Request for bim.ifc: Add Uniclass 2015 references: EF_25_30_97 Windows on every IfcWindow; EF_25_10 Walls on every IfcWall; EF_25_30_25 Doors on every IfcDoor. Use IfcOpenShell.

First a look at what the model holds.

```python
import ifcopenshell

model = ifcopenshell.open("bim.ifc")
print(model.schema)
print("classifications:", [c.Name for c in model.by_type("IfcClassification")])
for ifc_class in ("IfcDoor", "IfcRoof", "IfcStair", "IfcWall", "IfcWindow"):
    print(ifc_class, len(model.by_type(ifc_class)))
```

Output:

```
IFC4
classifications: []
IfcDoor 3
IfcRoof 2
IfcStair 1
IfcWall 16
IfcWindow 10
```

```python
import ifcopenshell
import ifcopenshell.api.classification

model = ifcopenshell.open("bim.ifc")

system = ifcopenshell.api.classification.add_classification(model, classification="Uniclass 2015")

codes = {
    "IfcWindow": ("EF_25_30_97", "Windows"),
    "IfcWall": ("EF_25_10", "Walls"),
    "IfcDoor": ("EF_25_30_25", "Doors"),
}
for ifc_class, (code, name) in codes.items():
    products = model.by_type(ifc_class)
    ifcopenshell.api.classification.add_reference(
        model, products=products, classification=system, identification=code, name=name
    )
    print(code, len(products))

model.write("bim_edited.ifc")
```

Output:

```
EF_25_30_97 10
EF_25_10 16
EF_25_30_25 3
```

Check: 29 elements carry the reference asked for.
